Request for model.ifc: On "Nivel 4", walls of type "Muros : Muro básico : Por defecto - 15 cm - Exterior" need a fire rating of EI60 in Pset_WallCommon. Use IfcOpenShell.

First a look at what the model holds.

```python
import ifcopenshell
import ifcopenshell.util.element

model = ifcopenshell.open("model.ifc")
print(model.schema)
storey = next(s for s in model.by_type("IfcBuildingStorey") if s.Name == "Nivel 4")
walls = [e for e in ifcopenshell.util.element.get_decomposition(storey) if e.is_a("IfcWall")]
seen = {}
for e in walls:
    element_type = ifcopenshell.util.element.get_type(e)
    key = (element_type.Name if element_type != e and element_type else None, ifcopenshell.util.element.get_pset(e, "Pset_WallCommon", "FireRating"))
    seen[key] = seen.get(key, 0) + 1
for (name, value), count in sorted(seen.items(), key=str):
    print(count, "x", name, "|", value)
```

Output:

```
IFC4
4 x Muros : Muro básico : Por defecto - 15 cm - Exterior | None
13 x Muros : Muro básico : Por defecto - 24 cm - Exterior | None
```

```python
import ifcopenshell
import ifcopenshell.api.pset
import ifcopenshell.util.element

model = ifcopenshell.open("model.ifc")

storey = next(s for s in model.by_type("IfcBuildingStorey") if s.Name == "Nivel 4")
walls = [e for e in ifcopenshell.util.element.get_decomposition(storey) if e.is_a("IfcWall")]

count = 0
for e in walls:
    element_type = ifcopenshell.util.element.get_type(e)
    if element_type in (None, e) or element_type.Name != "Muros : Muro básico : Por defecto - 15 cm - Exterior":
        continue
    # add_pset returns the element's existing set when there is one.
    pset = ifcopenshell.api.pset.add_pset(model, product=e, name="Pset_WallCommon")
    ifcopenshell.api.pset.edit_pset(model, pset=pset, properties={"FireRating": "EI60"})
    count += 1

print(count, "walls updated")

model.write("model_updated.ifc")
```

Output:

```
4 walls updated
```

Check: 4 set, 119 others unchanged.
